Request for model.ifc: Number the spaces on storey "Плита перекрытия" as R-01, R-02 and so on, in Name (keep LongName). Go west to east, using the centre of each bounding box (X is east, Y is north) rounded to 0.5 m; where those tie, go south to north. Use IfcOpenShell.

First a look at what the model holds.

```python
import ifcopenshell
import ifcopenshell.util.element
import ifcopenshell.util.placement

model = ifcopenshell.open("model.ifc")
print(model.schema)
storey = next(s for s in model.by_type("IfcBuildingStorey") if s.Name == "Плита перекрытия")
spaces = [e for e in ifcopenshell.util.element.get_decomposition(storey) if e.is_a("IfcSpace")]
for e in sorted(spaces, key=lambda e: e.id()):
    origin = ifcopenshell.util.placement.get_local_placement(e.ObjectPlacement)[:3, 3]
    print(e.id(), e.Name, e.LongName, origin.round(2) + 0.0, sep=" | ")
```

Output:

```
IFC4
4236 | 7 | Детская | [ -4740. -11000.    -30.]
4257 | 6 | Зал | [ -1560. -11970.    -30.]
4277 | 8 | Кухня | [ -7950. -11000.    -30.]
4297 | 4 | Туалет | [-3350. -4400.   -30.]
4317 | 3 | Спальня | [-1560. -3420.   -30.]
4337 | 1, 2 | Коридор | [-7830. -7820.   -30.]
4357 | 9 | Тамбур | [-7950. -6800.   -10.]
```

```python
import ifcopenshell
import ifcopenshell.geom
import ifcopenshell.util.element
import ifcopenshell.util.shape

model = ifcopenshell.open("model.ifc")
settings = ifcopenshell.geom.settings()
settings.set("use-world-coords", True)


def centre(element):
    shape = ifcopenshell.geom.create_shape(settings, element)
    return ifcopenshell.util.shape.get_bbox_centroid(shape.geometry)


storey = next(s for s in model.by_type("IfcBuildingStorey") if s.Name == "Плита перекрытия")
spaces = [e for e in ifcopenshell.util.element.get_decomposition(storey) if e.is_a("IfcSpace")]

# Insertion points can sit at a corner or the storey origin, so sort by the geometry (in metres).
centres = {e: centre(e) for e in spaces}
spaces.sort(key=lambda e: (round(centres[e][0] / 0.5), centres[e][1]))

for i, e in enumerate(spaces, start=1):
    number = f"R-{i:02d}"
    e.Name = number
    print(e.id(), number)

model.write("model_rev.ifc")
```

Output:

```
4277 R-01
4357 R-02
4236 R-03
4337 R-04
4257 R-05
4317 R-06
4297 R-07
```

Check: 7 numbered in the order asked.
